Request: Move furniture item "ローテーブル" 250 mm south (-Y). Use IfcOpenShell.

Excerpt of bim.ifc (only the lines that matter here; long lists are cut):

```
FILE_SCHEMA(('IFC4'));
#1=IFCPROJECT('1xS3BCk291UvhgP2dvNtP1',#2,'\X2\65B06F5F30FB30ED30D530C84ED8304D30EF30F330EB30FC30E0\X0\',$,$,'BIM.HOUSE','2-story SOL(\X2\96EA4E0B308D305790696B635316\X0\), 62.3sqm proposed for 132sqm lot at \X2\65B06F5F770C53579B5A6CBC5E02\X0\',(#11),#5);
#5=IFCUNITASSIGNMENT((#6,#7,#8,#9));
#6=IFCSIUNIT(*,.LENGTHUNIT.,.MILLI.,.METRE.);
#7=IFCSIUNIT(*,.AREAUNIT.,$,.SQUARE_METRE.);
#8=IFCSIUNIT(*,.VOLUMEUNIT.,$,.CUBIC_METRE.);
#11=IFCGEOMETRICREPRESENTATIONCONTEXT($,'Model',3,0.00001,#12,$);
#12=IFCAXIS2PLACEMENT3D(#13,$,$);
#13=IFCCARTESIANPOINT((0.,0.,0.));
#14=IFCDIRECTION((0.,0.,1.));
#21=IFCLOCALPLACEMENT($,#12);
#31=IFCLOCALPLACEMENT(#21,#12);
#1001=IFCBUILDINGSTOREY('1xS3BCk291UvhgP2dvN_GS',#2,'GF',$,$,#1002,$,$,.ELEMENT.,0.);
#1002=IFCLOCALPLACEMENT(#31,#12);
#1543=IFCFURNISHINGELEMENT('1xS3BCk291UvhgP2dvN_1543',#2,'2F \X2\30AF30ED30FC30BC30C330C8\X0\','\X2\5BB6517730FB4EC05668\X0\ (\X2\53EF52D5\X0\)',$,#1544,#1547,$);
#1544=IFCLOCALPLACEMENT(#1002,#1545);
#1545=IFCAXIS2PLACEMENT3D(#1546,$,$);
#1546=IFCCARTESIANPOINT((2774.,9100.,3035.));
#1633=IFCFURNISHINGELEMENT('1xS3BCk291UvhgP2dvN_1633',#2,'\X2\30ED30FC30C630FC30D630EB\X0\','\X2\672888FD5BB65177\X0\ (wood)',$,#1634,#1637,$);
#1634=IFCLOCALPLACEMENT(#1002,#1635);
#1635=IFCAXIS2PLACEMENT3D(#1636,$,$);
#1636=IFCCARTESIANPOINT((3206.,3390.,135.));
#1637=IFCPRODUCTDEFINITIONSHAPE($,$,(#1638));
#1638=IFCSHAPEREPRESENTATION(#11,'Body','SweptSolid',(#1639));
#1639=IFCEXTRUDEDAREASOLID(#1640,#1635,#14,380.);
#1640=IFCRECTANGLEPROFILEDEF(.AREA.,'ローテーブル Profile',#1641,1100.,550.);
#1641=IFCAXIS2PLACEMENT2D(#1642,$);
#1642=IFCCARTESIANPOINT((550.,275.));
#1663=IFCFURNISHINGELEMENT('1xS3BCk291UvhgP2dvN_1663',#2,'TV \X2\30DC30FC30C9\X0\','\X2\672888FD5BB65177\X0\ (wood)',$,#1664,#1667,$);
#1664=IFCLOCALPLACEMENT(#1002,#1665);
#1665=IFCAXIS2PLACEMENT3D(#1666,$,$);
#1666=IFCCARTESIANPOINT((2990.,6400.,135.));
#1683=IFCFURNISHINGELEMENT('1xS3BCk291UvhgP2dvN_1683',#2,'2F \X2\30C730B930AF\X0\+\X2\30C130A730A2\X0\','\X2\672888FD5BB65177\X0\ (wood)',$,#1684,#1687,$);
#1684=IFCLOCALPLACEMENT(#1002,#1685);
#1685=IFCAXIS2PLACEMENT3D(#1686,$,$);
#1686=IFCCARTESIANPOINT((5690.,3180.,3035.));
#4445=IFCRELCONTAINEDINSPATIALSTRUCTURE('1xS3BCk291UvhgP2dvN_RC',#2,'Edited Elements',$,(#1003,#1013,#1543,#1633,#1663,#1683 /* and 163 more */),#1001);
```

```python
import ifcopenshell
import ifcopenshell.api.geometry
import ifcopenshell.util.placement

model = ifcopenshell.open("bim.ifc")

item = model.by_guid("1xS3BCk291UvhgP2dvN_1633")
matrix = ifcopenshell.util.placement.get_local_placement(item.ObjectPlacement)
matrix[1, 3] -= 250.0
ifcopenshell.api.geometry.edit_object_placement(model, product=item, matrix=matrix, is_si=False)

print(ifcopenshell.util.placement.get_local_placement(item.ObjectPlacement).round(3) + 0.0)

model.write("bim_v2.ifc")
```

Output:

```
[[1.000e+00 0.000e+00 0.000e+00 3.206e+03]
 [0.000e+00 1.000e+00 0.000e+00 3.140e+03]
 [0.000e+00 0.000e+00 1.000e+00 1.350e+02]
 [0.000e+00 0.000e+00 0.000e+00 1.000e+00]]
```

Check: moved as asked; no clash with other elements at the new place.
